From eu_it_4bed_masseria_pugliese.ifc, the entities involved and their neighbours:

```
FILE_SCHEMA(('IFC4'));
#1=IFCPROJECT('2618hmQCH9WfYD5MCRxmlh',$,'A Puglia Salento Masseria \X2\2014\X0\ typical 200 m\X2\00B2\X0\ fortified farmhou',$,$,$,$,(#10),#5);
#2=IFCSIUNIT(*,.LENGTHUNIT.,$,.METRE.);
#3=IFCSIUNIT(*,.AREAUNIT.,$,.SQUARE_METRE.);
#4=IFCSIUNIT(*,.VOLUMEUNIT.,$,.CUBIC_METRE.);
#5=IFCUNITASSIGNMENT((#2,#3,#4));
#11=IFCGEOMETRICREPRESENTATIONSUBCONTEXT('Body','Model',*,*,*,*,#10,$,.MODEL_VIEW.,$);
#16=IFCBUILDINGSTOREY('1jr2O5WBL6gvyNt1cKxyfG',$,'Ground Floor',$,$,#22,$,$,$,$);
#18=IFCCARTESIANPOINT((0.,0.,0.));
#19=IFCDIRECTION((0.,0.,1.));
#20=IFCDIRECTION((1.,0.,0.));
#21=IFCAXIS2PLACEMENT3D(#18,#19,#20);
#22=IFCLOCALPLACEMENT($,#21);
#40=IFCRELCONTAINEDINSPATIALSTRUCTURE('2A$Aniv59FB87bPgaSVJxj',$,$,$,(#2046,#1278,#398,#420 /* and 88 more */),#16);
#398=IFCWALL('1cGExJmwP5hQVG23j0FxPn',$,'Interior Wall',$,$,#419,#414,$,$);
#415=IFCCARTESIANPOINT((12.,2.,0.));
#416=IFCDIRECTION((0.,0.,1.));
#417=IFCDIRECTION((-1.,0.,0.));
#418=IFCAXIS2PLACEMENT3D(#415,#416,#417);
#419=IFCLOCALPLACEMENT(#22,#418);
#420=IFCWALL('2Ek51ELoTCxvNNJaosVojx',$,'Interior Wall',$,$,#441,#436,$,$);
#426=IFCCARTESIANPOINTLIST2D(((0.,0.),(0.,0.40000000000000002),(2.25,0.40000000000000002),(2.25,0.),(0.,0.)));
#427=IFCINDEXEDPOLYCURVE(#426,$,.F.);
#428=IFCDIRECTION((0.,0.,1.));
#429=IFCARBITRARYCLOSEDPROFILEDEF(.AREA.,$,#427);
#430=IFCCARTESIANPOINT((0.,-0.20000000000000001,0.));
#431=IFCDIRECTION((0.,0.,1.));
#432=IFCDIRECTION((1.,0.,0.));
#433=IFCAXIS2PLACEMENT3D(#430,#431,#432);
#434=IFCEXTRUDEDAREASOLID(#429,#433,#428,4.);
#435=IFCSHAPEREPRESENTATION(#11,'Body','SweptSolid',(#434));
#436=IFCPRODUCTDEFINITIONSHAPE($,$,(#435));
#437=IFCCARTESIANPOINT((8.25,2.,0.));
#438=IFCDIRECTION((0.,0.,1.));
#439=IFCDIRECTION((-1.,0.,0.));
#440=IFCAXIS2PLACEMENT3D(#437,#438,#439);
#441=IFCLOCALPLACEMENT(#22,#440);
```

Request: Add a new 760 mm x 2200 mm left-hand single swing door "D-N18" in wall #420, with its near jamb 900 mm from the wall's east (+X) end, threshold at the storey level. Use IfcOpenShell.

```python
import numpy as np
import ifcopenshell
import ifcopenshell.api.feature
import ifcopenshell.api.geometry
import ifcopenshell.api.root
import ifcopenshell.api.spatial
import ifcopenshell.geom
import ifcopenshell.util.element
import ifcopenshell.util.placement
import ifcopenshell.util.representation
import ifcopenshell.util.shape
import ifcopenshell.util.unit

model = ifcopenshell.open("eu_it_4bed_masseria_pugliese.ifc")
unit_scale = ifcopenshell.util.unit.calculate_unit_scale(model)
settings = ifcopenshell.geom.settings()


def volume(element):
    """Net volume in cubic metres, openings subtracted."""
    shape = ifcopenshell.geom.create_shape(settings, element)
    return ifcopenshell.util.shape.get_volume(shape.geometry)


wall = model.by_guid("2Ek51ELoTCxvNNJaosVojx")
storey = ifcopenshell.util.element.get_container(wall, ifc_class="IfcBuildingStorey")
context = ifcopenshell.util.representation.get_context(model, "Model", "Body", "MODEL_VIEW")
before = volume(wall)

width, height, from_end, sill = 0.76, 2.2, 0.9, 0.0  # metres

# The wall runs along its own X axis, and the end named is its -X end.
wall_shape = ifcopenshell.geom.create_shape(settings, wall)
x, y, z = ifcopenshell.util.shape.get_vertices(wall_shape.geometry).T
start = x.min() + from_end
face, thickness = float(y.min()), float(y.max() - y.min())
wall_matrix = ifcopenshell.util.placement.get_local_placement(wall.ObjectPlacement)
level = ifcopenshell.util.placement.get_local_placement(storey.ObjectPlacement)[2, 3]


def in_wall(x, y):
    """Placement at x, y metres in the wall's axes, at sill height."""
    matrix = wall_matrix.copy()
    matrix[:, 3] = wall_matrix @ np.array([x / unit_scale, y / unit_scale, 0.0, 1.0])
    matrix[2, 3] = level + sill / unit_scale
    return matrix


# Opening: a box that overshoots both wall faces by 50 mm.
opening = ifcopenshell.api.root.create_entity(model, ifc_class="IfcOpeningElement", predefined_type="OPENING")
box = ifcopenshell.api.geometry.add_wall_representation(
    model, context=context, length=width, height=height, thickness=thickness + 0.1
)
ifcopenshell.api.geometry.assign_representation(model, product=opening, representation=box)
ifcopenshell.api.geometry.edit_object_placement(model, product=opening, matrix=in_wall(start, face - 0.05), is_si=False)
ifcopenshell.api.feature.add_feature(model, feature=opening, element=wall)

door = ifcopenshell.api.root.create_entity(model, ifc_class="IfcDoor", name="D-N18", predefined_type="DOOR")
door.OverallWidth, door.OverallHeight = width / unit_scale, height / unit_scale
door.OperationType = "SINGLE_SWING_LEFT"
body = ifcopenshell.api.geometry.add_door_representation(
    model,
    context=context,
    overall_width=door.OverallWidth,
    overall_height=door.OverallHeight,
    operation_type="SINGLE_SWING_LEFT",
    lining_properties={"LiningDepth": thickness / unit_scale, "ThresholdDepth": thickness / unit_scale},
)
ifcopenshell.api.geometry.assign_representation(model, product=door, representation=body)
ifcopenshell.api.spatial.assign_container(model, products=[door], relating_structure=storey)
ifcopenshell.api.feature.add_filling(model, opening=opening, element=door)

# The lining spans the wall, so the door starts at the wall face.
ifcopenshell.api.geometry.edit_object_placement(model, product=door, matrix=in_wall(start, face), is_si=False)

after = volume(wall)

print(f"wall volume {before:.3f} -> {after:.3f} m3")

model.write("eu_it_4bed_masseria_pugliese_rev.ifc")
```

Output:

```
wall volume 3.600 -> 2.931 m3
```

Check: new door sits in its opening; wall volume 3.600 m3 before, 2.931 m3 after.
